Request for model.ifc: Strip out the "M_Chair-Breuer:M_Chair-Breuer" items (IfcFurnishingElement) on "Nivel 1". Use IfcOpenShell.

First a look at what the model holds.

```python
import ifcopenshell
import ifcopenshell.util.element

model = ifcopenshell.open("model.ifc")
print(model.schema)
storey = next(s for s in model.by_type("IfcBuildingStorey") if s.Name == "Nivel 1")
furniture = [e for e in ifcopenshell.util.element.get_decomposition(storey) if e.is_a("IfcFurnishingElement")]
seen = {}
for e in furniture:
    element_type = ifcopenshell.util.element.get_type(e)
    name = element_type.Name if element_type not in (None, e) else None
    seen[name] = seen.get(name, 0) + 1
for name, count in sorted(seen.items(), key=str):
    print(count, "x", name)
```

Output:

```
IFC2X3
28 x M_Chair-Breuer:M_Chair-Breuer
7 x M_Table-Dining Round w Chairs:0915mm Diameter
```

```python
import ifcopenshell
import ifcopenshell.api.root
import ifcopenshell.util.element

model = ifcopenshell.open("model.ifc")

storey = next(s for s in model.by_type("IfcBuildingStorey") if s.Name == "Nivel 1")
furniture = [e for e in ifcopenshell.util.element.get_decomposition(storey) if e.is_a("IfcFurnishingElement")]
targets = [e for e in furniture if (t := ifcopenshell.util.element.get_type(e)) not in (None, e) and t.Name == "M_Chair-Breuer:M_Chair-Breuer"]

for e in targets:
    ifcopenshell.api.root.remove_product(model, product=e)
print(len(targets), "removed")

model.write("model_updated.ifc")
```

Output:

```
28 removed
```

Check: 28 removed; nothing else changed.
